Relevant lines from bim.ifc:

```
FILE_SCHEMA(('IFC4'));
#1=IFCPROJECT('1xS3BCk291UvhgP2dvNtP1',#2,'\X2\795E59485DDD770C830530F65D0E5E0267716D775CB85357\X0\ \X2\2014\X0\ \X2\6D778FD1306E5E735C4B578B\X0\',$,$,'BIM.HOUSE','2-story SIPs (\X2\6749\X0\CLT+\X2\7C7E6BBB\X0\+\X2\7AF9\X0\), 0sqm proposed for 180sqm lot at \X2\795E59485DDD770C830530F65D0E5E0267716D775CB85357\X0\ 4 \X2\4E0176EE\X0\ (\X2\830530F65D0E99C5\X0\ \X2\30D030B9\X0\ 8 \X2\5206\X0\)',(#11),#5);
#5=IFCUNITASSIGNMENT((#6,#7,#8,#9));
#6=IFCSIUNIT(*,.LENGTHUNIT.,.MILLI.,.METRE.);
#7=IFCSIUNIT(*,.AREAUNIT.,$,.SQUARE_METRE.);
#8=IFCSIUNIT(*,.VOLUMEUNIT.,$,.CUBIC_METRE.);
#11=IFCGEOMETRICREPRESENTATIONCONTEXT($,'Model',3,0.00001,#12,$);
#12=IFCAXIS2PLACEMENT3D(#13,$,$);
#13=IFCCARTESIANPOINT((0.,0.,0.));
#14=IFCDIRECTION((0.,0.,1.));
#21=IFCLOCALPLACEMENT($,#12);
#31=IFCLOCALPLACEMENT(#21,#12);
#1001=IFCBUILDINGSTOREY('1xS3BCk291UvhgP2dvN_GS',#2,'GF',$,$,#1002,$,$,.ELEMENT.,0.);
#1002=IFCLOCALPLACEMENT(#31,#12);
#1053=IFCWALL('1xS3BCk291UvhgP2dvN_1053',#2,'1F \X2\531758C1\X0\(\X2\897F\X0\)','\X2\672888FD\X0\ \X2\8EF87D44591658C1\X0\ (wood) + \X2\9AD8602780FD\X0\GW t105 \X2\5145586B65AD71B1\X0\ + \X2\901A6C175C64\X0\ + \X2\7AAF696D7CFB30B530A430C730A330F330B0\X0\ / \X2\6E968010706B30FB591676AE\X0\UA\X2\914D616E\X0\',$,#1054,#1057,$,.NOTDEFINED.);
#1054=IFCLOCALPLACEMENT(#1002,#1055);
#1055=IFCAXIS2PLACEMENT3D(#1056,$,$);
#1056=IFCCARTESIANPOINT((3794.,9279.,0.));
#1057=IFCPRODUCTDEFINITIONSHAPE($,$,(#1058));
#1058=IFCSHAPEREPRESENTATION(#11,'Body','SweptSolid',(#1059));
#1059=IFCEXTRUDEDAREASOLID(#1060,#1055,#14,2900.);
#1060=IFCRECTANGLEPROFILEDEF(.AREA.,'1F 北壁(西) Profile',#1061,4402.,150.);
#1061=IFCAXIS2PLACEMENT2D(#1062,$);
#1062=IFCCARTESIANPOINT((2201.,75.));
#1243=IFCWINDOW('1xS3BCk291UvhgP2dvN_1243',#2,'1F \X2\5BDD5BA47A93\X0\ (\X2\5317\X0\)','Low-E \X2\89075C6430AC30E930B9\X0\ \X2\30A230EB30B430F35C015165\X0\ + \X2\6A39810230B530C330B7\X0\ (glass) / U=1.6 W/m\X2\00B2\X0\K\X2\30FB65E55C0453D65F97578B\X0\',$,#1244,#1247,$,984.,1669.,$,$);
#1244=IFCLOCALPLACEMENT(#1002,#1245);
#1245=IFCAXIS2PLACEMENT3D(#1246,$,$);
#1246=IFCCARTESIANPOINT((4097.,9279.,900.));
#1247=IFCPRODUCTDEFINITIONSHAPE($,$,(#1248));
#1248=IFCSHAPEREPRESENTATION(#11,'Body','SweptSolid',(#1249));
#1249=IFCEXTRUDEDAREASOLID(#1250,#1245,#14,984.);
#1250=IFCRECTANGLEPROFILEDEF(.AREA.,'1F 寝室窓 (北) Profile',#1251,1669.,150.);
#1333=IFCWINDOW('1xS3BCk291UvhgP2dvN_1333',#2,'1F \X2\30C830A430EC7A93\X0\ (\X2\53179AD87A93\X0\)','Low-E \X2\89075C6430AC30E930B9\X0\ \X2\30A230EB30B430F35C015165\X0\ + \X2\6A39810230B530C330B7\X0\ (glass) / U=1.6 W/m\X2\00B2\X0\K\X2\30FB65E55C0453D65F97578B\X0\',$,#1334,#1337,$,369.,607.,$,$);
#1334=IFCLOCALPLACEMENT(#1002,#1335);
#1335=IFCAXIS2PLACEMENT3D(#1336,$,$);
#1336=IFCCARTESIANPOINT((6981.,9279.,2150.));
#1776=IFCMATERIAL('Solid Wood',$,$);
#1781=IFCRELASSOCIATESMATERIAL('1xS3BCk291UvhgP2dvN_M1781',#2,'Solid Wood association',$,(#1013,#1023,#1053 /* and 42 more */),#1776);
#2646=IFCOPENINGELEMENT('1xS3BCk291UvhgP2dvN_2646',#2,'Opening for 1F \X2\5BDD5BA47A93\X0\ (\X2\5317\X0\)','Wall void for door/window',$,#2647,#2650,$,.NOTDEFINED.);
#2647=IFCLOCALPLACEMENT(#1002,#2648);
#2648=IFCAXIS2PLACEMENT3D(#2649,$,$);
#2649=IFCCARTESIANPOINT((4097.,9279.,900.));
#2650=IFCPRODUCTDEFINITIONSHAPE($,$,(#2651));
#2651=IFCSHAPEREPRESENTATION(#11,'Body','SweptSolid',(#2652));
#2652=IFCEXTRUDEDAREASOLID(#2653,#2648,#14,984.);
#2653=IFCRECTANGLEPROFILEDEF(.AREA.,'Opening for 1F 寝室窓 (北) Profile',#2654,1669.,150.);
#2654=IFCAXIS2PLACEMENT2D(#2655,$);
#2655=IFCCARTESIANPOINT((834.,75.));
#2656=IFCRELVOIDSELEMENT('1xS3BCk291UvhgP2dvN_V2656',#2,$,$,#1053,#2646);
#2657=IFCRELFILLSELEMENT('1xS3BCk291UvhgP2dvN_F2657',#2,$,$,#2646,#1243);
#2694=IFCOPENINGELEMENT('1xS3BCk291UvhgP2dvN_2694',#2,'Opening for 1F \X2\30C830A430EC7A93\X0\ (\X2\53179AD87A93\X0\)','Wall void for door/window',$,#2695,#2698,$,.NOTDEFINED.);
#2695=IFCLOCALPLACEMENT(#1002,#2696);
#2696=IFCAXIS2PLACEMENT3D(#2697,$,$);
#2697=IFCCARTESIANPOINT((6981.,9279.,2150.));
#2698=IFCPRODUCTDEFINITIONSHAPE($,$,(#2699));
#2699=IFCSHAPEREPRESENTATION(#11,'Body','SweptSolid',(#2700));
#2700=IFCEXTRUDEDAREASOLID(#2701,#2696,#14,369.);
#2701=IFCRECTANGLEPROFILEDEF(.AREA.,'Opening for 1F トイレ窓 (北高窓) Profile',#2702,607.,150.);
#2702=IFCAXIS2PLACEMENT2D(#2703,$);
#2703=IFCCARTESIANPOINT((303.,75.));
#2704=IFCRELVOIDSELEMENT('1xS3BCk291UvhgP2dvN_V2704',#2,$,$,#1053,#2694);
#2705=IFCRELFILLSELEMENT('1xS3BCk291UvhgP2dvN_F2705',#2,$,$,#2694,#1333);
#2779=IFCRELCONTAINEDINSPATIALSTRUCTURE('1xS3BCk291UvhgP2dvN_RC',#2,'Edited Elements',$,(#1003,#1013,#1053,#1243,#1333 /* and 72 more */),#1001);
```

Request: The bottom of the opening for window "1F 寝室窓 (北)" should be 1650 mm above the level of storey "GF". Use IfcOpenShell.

```python
import numpy as np
import ifcopenshell
import ifcopenshell.api.geometry
import ifcopenshell.geom
import ifcopenshell.util.element
import ifcopenshell.util.placement
import ifcopenshell.util.shape
import ifcopenshell.util.unit

model = ifcopenshell.open("bim.ifc")
unit_scale = ifcopenshell.util.unit.calculate_unit_scale(model)

window = model.by_guid("1xS3BCk291UvhgP2dvN_1243")
opening = window.FillsVoids[0].RelatingOpeningElement
storey = ifcopenshell.util.element.get_container(window, ifc_class="IfcBuildingStorey")
level = ifcopenshell.util.placement.get_local_placement(storey.ObjectPlacement)[2, 3]

# The opening's origin need not be at the sill, so measure its lowest point.
shape = ifcopenshell.geom.create_shape(ifcopenshell.geom.settings(), opening)
bottom = ifcopenshell.util.shape.get_shape_bottom_elevation(shape, shape.geometry) / unit_scale
dz = level + 1650.0 - bottom

shift = np.array([0.0, 0.0, dz])
# The window is not placed relative to its opening, so move both.
for product in (opening, window):
    matrix = ifcopenshell.util.placement.get_local_placement(product.ObjectPlacement)
    matrix[:3, 3] += shift
    ifcopenshell.api.geometry.edit_object_placement(model, product=product, matrix=matrix, is_si=False)

print(f"moved by {dz * unit_scale:+.3f} m")

model.write("bim-out.ifc")
```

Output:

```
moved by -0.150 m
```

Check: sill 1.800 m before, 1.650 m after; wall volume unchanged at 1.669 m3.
